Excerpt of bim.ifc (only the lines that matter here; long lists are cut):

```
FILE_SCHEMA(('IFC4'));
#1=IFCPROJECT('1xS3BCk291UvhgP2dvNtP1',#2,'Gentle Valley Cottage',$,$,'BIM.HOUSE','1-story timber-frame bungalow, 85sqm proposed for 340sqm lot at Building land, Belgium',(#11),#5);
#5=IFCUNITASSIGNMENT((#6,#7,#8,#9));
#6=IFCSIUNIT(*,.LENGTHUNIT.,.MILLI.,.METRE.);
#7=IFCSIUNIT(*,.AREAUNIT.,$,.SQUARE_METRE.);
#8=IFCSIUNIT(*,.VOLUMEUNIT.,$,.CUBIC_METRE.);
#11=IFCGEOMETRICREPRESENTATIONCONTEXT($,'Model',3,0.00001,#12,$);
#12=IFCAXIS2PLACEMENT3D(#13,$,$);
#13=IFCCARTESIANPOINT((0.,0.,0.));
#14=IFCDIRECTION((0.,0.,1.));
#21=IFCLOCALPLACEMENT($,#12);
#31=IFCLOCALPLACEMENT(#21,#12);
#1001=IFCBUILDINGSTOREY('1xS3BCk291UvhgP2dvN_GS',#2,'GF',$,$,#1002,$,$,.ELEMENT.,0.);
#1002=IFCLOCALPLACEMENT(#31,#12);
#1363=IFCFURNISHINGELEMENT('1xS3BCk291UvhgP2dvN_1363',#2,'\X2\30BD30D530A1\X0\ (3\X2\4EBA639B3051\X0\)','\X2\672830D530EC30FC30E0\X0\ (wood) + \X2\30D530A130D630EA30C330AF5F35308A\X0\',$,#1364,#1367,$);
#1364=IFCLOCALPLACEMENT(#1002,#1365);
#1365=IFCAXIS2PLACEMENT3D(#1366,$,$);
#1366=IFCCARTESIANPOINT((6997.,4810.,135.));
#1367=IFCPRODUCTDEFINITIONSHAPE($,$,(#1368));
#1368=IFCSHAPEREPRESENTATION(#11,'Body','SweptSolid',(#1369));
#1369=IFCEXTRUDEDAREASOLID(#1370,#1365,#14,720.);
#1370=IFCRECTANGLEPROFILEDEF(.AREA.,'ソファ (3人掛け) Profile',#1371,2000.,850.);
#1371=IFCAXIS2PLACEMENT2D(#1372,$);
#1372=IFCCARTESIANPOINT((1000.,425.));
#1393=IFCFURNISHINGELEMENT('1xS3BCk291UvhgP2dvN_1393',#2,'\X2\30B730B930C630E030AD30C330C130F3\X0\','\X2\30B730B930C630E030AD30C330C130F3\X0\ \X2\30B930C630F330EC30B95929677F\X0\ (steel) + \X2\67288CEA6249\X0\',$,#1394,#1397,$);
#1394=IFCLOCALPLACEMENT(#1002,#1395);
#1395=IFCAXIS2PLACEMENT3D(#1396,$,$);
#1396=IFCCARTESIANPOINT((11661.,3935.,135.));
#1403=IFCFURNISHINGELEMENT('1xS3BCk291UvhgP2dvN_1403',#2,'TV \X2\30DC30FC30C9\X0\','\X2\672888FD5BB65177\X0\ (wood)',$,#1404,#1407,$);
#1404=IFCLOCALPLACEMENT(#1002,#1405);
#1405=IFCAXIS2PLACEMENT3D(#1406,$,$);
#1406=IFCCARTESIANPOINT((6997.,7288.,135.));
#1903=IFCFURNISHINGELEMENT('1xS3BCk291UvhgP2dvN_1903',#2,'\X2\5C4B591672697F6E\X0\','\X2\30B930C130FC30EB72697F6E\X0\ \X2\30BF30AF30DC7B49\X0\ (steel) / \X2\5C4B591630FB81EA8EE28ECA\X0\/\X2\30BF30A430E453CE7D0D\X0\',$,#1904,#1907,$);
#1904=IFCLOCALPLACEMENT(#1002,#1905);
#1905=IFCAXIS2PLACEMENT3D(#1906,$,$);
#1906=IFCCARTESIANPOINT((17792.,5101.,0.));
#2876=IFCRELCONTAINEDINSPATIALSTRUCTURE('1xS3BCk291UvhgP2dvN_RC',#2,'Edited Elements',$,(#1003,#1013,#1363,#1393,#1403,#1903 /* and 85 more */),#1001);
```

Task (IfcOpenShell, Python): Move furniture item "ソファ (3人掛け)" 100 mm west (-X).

```python
import ifcopenshell
import ifcopenshell.api.geometry
import ifcopenshell.util.placement

model = ifcopenshell.open("bim.ifc")

item = model.by_guid("1xS3BCk291UvhgP2dvN_1363")
matrix = ifcopenshell.util.placement.get_local_placement(item.ObjectPlacement)
matrix[0, 3] -= 100.0
ifcopenshell.api.geometry.edit_object_placement(model, product=item, matrix=matrix, is_si=False)

print(ifcopenshell.util.placement.get_local_placement(item.ObjectPlacement).round(3) + 0.0)

model.write("bim_v2.ifc")
```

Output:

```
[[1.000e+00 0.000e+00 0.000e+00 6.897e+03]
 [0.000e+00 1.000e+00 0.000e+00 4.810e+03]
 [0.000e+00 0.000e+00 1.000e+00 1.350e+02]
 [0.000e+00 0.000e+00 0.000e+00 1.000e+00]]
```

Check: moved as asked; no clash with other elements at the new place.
